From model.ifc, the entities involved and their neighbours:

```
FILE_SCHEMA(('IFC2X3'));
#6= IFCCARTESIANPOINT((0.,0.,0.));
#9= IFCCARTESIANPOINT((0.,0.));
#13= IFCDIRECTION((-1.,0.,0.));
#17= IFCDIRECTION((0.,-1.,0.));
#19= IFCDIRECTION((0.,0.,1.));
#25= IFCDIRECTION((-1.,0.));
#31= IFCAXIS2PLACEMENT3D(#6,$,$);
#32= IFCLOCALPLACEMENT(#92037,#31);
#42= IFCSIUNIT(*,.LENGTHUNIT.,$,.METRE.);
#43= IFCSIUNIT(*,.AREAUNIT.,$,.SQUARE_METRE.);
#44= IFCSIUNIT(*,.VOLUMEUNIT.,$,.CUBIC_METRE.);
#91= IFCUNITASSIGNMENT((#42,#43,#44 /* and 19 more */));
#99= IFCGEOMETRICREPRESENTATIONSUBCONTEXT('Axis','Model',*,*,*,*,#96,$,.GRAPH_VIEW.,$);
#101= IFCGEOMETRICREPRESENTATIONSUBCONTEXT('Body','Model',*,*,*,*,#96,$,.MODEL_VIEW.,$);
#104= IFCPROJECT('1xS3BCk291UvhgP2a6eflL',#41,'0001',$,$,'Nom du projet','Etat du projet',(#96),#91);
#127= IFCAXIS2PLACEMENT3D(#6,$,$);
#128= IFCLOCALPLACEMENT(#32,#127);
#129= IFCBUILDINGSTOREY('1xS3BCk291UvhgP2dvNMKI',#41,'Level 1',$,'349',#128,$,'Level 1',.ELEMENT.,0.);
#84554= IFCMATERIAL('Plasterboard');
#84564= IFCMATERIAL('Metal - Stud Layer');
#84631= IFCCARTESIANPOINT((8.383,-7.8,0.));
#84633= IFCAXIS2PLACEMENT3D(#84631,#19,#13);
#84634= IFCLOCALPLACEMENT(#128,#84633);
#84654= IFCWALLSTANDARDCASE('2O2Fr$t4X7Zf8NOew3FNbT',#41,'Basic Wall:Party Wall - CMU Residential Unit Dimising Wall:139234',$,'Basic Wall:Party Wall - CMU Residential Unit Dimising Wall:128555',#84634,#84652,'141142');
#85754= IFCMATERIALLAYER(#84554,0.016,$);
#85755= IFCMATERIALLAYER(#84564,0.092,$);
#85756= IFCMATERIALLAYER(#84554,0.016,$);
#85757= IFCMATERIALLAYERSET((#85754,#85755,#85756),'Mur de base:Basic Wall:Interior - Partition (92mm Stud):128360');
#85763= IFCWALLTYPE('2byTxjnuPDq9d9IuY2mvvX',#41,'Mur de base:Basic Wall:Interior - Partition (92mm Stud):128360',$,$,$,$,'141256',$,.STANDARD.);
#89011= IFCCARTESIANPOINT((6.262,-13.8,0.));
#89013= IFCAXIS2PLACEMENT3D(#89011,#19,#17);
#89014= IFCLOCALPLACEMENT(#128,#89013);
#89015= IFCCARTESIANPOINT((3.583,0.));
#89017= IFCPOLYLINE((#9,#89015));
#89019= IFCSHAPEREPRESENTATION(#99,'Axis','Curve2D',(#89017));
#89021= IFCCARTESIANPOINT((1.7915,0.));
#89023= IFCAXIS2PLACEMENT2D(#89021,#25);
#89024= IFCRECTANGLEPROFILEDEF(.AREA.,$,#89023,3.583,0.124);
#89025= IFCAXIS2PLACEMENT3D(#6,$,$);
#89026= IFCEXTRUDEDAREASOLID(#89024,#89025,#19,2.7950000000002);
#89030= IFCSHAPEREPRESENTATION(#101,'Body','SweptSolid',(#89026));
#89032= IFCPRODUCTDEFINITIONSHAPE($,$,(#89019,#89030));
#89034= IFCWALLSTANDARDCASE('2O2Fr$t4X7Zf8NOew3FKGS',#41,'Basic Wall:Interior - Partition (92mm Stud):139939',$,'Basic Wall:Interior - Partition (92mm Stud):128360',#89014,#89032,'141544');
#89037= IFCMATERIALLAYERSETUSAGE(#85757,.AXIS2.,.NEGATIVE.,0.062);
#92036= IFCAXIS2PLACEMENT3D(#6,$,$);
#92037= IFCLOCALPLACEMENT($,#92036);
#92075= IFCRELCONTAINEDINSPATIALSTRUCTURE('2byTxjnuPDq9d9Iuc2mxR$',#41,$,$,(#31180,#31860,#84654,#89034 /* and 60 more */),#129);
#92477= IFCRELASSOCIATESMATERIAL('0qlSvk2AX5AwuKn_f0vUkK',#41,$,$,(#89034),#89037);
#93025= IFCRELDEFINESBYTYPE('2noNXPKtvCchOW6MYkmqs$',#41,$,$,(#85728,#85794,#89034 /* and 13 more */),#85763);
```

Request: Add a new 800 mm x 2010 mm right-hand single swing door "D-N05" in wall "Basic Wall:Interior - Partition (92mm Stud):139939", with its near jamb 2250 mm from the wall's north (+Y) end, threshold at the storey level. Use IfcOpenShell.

```python
import numpy as np
import ifcopenshell
import ifcopenshell.api.feature
import ifcopenshell.api.geometry
import ifcopenshell.api.root
import ifcopenshell.api.spatial
import ifcopenshell.api.type
import ifcopenshell.geom
import ifcopenshell.util.element
import ifcopenshell.util.placement
import ifcopenshell.util.representation
import ifcopenshell.util.shape
import ifcopenshell.util.unit

model = ifcopenshell.open("model.ifc")
unit_scale = ifcopenshell.util.unit.calculate_unit_scale(model)
settings = ifcopenshell.geom.settings()


def volume(element):
    """Net volume in cubic metres, openings subtracted."""
    shape = ifcopenshell.geom.create_shape(settings, element)
    return ifcopenshell.util.shape.get_volume(shape.geometry)


wall = model.by_id(89034)
storey = ifcopenshell.util.element.get_container(wall, ifc_class="IfcBuildingStorey")
context = ifcopenshell.util.representation.get_context(model, "Model", "Body", "MODEL_VIEW")
before = volume(wall)

width, height, from_end, sill = 0.8, 2.01, 2.25, 0.0  # metres

# The wall runs along its own X axis, and the end named is its -X end.
wall_shape = ifcopenshell.geom.create_shape(settings, wall)
x, y, z = ifcopenshell.util.shape.get_vertices(wall_shape.geometry).T
start = x.min() + from_end
face, thickness = float(y.min()), float(y.max() - y.min())
wall_matrix = ifcopenshell.util.placement.get_local_placement(wall.ObjectPlacement)
level = ifcopenshell.util.placement.get_local_placement(storey.ObjectPlacement)[2, 3]


def in_wall(x, y):
    """Placement at x, y metres in the wall's axes, at sill height."""
    matrix = wall_matrix.copy()
    matrix[:, 3] = wall_matrix @ np.array([x / unit_scale, y / unit_scale, 0.0, 1.0])
    matrix[2, 3] = level + sill / unit_scale
    return matrix


# Opening: a box that overshoots both wall faces by 50 mm.
opening = ifcopenshell.api.root.create_entity(model, ifc_class="IfcOpeningElement")
box = ifcopenshell.api.geometry.add_wall_representation(
    model, context=context, length=width, height=height, thickness=thickness + 0.1
)
ifcopenshell.api.geometry.assign_representation(model, product=opening, representation=box)
ifcopenshell.api.geometry.edit_object_placement(model, product=opening, matrix=in_wall(start, face - 0.05), is_si=False)
ifcopenshell.api.feature.add_feature(model, feature=opening, element=wall)

door = ifcopenshell.api.root.create_entity(model, ifc_class="IfcDoor", name="D-N05")
door.OverallWidth, door.OverallHeight = width / unit_scale, height / unit_scale
body = ifcopenshell.api.geometry.add_door_representation(
    model,
    context=context,
    overall_width=door.OverallWidth,
    overall_height=door.OverallHeight,
    operation_type="SINGLE_SWING_RIGHT",
    lining_properties={"LiningDepth": thickness / unit_scale, "ThresholdDepth": thickness / unit_scale},
)
ifcopenshell.api.geometry.assign_representation(model, product=door, representation=body)
ifcopenshell.api.spatial.assign_container(model, products=[door], relating_structure=storey)
fills = ifcopenshell.api.feature.add_filling(model, opening=opening, element=door)
fills.OwnerHistory = door.OwnerHistory  # required in IFC2X3

# IFC2X3 keeps the operation on the door style.
style = ifcopenshell.api.root.create_entity(model, ifc_class="IfcDoorStyle", name="D-N05")
style.OperationType, style.ConstructionType = "SINGLE_SWING_RIGHT", "NOTDEFINED"
style.ParameterTakesPrecedence = style.Sizeable = False
ifcopenshell.api.type.assign_type(model, related_objects=[door], relating_type=style)

# The lining spans the wall, so the door starts at the wall face.
ifcopenshell.api.geometry.edit_object_placement(model, product=door, matrix=in_wall(start, face), is_si=False)

after = volume(wall)

print(f"wall volume {before:.3f} -> {after:.3f} m3")

model.write("model_updated.ifc")
```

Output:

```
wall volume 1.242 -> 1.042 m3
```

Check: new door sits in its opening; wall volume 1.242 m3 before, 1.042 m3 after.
